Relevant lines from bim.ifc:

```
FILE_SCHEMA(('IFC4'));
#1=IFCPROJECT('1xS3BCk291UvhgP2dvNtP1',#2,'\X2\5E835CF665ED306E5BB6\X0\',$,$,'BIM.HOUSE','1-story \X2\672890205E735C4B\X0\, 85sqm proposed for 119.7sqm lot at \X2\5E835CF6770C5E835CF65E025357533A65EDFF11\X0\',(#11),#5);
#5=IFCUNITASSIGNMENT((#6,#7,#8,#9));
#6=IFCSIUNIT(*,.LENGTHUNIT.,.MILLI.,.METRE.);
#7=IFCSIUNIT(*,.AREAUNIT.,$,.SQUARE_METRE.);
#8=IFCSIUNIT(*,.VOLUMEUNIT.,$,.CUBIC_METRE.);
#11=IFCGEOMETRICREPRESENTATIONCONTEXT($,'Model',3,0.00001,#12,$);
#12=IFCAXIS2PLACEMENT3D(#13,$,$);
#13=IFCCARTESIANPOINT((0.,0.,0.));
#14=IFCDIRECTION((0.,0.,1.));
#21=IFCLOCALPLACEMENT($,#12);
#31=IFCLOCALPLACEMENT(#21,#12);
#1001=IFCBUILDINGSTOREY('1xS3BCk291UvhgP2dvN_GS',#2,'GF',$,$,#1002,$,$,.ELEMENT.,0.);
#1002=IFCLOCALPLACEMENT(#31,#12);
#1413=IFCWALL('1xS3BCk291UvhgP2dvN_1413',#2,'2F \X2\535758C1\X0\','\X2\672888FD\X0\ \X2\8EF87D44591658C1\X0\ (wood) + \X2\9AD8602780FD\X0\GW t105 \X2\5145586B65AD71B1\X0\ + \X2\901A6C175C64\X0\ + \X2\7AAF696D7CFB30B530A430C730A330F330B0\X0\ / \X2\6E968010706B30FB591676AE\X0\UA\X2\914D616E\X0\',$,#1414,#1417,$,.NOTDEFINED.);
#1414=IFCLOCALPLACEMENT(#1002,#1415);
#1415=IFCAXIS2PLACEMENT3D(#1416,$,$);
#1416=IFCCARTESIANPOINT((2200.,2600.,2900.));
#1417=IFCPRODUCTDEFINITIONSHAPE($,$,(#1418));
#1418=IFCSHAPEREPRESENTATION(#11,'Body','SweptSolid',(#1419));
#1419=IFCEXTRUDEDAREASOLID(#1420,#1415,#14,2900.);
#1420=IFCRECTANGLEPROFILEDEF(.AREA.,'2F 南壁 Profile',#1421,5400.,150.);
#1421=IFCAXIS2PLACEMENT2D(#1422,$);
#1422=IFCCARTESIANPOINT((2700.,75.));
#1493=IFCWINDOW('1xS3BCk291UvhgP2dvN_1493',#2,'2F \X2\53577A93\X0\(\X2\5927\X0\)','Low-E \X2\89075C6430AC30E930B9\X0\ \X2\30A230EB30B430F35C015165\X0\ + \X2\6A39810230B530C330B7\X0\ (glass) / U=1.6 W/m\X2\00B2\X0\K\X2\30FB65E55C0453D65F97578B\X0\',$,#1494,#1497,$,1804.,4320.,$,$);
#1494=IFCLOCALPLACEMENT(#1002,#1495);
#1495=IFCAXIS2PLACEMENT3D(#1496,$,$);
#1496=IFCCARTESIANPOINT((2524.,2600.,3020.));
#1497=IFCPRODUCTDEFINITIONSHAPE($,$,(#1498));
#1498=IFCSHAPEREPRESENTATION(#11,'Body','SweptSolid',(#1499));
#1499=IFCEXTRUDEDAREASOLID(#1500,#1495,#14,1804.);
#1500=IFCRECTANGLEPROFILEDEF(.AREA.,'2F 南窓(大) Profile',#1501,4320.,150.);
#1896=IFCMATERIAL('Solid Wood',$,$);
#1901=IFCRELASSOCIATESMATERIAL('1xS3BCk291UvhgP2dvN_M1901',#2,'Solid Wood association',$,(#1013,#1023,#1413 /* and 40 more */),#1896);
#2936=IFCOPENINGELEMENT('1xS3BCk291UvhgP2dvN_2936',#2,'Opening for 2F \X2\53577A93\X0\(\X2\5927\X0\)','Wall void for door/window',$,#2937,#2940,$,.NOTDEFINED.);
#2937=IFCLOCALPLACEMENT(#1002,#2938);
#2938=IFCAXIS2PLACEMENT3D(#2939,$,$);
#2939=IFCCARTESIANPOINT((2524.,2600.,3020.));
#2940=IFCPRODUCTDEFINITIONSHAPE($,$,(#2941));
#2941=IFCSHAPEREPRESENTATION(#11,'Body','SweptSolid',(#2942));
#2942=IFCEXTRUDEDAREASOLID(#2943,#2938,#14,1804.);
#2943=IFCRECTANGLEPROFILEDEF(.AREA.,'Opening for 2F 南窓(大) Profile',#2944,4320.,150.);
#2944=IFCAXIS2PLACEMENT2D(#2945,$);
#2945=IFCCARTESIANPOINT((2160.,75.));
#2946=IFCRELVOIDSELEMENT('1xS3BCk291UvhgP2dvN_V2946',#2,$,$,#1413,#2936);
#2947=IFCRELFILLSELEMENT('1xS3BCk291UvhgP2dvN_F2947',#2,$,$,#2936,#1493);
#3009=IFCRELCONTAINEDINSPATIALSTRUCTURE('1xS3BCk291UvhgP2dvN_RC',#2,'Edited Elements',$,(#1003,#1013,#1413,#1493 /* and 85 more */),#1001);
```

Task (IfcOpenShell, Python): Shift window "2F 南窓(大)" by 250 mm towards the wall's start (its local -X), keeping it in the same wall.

```python
import ifcopenshell
import ifcopenshell.api.geometry
import ifcopenshell.util.placement
import ifcopenshell.util.unit

model = ifcopenshell.open("bim.ifc")
unit_scale = ifcopenshell.util.unit.calculate_unit_scale(model)

window = model.by_id(1493)
opening = window.FillsVoids[0].RelatingOpeningElement
wall = opening.VoidsElements[0].RelatingBuildingElement

wall_matrix = ifcopenshell.util.placement.get_local_placement(wall.ObjectPlacement)
shift = wall_matrix[:3, 0] * -0.25 / unit_scale
before = ifcopenshell.util.placement.get_local_placement(window.ObjectPlacement)[:3, 3].copy()

# The window is not placed relative to its opening, so move both.
for product in (opening, window):
    matrix = ifcopenshell.util.placement.get_local_placement(product.ObjectPlacement)
    matrix[:3, 3] += shift
    ifcopenshell.api.geometry.edit_object_placement(model, product=product, matrix=matrix, is_si=False)

after = ifcopenshell.util.placement.get_local_placement(window.ObjectPlacement)[:3, 3]
print("window moved by", (after - before).round(3) + 0.0)

model.write("bim_v2.ifc")
```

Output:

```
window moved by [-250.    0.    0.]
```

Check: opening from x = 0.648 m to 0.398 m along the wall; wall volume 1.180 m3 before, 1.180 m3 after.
